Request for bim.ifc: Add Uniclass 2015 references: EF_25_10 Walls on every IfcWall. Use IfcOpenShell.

First a look at what the model holds.

```python
import ifcopenshell

model = ifcopenshell.open("bim.ifc")
print(model.schema)
print("classifications:", [c.Name for c in model.by_type("IfcClassification")])
for ifc_class in ("IfcDoor", "IfcRoof", "IfcStair", "IfcWall", "IfcWindow"):
    print(ifc_class, len(model.by_type(ifc_class)))
```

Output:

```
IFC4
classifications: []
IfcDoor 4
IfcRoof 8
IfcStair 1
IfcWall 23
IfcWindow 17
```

```python
import ifcopenshell
import ifcopenshell.api.classification

model = ifcopenshell.open("bim.ifc")

system = ifcopenshell.api.classification.add_classification(model, classification="Uniclass 2015")

codes = {
    "IfcWall": ("EF_25_10", "Walls"),
}
for ifc_class, (code, name) in codes.items():
    products = model.by_type(ifc_class)
    ifcopenshell.api.classification.add_reference(
        model, products=products, classification=system, identification=code, name=name
    )
    print(code, len(products))

model.write("bim-out.ifc")
```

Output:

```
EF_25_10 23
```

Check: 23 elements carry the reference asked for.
